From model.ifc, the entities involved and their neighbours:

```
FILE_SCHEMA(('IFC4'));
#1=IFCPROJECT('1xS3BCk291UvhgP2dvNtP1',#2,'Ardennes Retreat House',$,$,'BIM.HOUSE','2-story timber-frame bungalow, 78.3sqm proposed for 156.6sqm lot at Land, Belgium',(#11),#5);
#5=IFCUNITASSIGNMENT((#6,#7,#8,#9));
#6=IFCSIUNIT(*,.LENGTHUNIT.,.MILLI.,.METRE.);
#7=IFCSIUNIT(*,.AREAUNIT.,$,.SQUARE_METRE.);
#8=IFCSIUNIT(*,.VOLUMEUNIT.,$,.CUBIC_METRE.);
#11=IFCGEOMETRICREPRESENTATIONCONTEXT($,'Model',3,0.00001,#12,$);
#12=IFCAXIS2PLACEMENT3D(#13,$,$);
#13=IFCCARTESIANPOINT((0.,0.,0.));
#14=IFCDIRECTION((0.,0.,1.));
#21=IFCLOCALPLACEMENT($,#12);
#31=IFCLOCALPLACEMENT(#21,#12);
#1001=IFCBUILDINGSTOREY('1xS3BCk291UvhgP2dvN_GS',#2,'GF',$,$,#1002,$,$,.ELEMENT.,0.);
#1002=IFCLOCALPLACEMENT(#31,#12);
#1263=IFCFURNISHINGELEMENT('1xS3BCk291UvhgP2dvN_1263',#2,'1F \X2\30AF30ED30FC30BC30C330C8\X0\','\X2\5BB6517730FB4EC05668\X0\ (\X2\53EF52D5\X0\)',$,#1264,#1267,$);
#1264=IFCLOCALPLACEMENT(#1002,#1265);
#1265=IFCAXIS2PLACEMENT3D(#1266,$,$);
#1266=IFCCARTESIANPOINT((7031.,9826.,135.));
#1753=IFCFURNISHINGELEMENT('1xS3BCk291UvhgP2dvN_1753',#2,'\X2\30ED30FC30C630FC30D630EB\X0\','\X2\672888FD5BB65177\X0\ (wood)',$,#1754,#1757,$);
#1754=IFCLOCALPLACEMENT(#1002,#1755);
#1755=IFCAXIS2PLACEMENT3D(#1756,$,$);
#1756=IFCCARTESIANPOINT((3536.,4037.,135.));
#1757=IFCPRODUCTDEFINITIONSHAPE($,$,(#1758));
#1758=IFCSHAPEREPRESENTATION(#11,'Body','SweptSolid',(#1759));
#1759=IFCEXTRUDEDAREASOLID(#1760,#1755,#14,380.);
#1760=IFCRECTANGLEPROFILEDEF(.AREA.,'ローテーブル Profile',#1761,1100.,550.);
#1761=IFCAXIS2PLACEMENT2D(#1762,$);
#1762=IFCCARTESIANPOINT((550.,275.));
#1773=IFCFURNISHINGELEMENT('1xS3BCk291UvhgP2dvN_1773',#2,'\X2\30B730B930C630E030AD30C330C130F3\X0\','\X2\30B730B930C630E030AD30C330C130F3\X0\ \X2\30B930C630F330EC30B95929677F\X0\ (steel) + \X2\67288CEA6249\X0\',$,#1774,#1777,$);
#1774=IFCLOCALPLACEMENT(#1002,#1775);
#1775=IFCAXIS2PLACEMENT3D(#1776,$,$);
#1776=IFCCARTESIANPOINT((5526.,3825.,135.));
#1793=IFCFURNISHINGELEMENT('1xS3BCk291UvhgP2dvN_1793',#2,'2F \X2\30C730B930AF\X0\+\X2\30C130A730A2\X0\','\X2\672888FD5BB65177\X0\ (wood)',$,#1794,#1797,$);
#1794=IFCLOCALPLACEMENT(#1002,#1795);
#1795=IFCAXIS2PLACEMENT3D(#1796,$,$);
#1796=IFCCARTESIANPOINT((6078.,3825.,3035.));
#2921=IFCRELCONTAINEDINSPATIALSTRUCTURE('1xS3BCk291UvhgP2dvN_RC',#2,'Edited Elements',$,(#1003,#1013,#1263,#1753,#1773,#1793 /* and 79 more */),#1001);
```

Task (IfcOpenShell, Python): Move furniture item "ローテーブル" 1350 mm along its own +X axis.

```python
import ifcopenshell
import ifcopenshell.api.geometry
import ifcopenshell.util.placement

model = ifcopenshell.open("model.ifc")

item = model.by_guid("1xS3BCk291UvhgP2dvN_1753")
matrix = ifcopenshell.util.placement.get_local_placement(item.ObjectPlacement)
matrix[:3, 3] += matrix[:3, 0] * 1350.0
ifcopenshell.api.geometry.edit_object_placement(model, product=item, matrix=matrix, is_si=False)

print(ifcopenshell.util.placement.get_local_placement(item.ObjectPlacement).round(3) + 0.0)

model.write("model_updated.ifc")
```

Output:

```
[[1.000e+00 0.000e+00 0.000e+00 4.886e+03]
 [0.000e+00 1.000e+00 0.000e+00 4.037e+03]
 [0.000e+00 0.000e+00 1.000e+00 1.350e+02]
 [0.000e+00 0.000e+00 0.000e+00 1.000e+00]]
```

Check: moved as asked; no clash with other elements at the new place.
